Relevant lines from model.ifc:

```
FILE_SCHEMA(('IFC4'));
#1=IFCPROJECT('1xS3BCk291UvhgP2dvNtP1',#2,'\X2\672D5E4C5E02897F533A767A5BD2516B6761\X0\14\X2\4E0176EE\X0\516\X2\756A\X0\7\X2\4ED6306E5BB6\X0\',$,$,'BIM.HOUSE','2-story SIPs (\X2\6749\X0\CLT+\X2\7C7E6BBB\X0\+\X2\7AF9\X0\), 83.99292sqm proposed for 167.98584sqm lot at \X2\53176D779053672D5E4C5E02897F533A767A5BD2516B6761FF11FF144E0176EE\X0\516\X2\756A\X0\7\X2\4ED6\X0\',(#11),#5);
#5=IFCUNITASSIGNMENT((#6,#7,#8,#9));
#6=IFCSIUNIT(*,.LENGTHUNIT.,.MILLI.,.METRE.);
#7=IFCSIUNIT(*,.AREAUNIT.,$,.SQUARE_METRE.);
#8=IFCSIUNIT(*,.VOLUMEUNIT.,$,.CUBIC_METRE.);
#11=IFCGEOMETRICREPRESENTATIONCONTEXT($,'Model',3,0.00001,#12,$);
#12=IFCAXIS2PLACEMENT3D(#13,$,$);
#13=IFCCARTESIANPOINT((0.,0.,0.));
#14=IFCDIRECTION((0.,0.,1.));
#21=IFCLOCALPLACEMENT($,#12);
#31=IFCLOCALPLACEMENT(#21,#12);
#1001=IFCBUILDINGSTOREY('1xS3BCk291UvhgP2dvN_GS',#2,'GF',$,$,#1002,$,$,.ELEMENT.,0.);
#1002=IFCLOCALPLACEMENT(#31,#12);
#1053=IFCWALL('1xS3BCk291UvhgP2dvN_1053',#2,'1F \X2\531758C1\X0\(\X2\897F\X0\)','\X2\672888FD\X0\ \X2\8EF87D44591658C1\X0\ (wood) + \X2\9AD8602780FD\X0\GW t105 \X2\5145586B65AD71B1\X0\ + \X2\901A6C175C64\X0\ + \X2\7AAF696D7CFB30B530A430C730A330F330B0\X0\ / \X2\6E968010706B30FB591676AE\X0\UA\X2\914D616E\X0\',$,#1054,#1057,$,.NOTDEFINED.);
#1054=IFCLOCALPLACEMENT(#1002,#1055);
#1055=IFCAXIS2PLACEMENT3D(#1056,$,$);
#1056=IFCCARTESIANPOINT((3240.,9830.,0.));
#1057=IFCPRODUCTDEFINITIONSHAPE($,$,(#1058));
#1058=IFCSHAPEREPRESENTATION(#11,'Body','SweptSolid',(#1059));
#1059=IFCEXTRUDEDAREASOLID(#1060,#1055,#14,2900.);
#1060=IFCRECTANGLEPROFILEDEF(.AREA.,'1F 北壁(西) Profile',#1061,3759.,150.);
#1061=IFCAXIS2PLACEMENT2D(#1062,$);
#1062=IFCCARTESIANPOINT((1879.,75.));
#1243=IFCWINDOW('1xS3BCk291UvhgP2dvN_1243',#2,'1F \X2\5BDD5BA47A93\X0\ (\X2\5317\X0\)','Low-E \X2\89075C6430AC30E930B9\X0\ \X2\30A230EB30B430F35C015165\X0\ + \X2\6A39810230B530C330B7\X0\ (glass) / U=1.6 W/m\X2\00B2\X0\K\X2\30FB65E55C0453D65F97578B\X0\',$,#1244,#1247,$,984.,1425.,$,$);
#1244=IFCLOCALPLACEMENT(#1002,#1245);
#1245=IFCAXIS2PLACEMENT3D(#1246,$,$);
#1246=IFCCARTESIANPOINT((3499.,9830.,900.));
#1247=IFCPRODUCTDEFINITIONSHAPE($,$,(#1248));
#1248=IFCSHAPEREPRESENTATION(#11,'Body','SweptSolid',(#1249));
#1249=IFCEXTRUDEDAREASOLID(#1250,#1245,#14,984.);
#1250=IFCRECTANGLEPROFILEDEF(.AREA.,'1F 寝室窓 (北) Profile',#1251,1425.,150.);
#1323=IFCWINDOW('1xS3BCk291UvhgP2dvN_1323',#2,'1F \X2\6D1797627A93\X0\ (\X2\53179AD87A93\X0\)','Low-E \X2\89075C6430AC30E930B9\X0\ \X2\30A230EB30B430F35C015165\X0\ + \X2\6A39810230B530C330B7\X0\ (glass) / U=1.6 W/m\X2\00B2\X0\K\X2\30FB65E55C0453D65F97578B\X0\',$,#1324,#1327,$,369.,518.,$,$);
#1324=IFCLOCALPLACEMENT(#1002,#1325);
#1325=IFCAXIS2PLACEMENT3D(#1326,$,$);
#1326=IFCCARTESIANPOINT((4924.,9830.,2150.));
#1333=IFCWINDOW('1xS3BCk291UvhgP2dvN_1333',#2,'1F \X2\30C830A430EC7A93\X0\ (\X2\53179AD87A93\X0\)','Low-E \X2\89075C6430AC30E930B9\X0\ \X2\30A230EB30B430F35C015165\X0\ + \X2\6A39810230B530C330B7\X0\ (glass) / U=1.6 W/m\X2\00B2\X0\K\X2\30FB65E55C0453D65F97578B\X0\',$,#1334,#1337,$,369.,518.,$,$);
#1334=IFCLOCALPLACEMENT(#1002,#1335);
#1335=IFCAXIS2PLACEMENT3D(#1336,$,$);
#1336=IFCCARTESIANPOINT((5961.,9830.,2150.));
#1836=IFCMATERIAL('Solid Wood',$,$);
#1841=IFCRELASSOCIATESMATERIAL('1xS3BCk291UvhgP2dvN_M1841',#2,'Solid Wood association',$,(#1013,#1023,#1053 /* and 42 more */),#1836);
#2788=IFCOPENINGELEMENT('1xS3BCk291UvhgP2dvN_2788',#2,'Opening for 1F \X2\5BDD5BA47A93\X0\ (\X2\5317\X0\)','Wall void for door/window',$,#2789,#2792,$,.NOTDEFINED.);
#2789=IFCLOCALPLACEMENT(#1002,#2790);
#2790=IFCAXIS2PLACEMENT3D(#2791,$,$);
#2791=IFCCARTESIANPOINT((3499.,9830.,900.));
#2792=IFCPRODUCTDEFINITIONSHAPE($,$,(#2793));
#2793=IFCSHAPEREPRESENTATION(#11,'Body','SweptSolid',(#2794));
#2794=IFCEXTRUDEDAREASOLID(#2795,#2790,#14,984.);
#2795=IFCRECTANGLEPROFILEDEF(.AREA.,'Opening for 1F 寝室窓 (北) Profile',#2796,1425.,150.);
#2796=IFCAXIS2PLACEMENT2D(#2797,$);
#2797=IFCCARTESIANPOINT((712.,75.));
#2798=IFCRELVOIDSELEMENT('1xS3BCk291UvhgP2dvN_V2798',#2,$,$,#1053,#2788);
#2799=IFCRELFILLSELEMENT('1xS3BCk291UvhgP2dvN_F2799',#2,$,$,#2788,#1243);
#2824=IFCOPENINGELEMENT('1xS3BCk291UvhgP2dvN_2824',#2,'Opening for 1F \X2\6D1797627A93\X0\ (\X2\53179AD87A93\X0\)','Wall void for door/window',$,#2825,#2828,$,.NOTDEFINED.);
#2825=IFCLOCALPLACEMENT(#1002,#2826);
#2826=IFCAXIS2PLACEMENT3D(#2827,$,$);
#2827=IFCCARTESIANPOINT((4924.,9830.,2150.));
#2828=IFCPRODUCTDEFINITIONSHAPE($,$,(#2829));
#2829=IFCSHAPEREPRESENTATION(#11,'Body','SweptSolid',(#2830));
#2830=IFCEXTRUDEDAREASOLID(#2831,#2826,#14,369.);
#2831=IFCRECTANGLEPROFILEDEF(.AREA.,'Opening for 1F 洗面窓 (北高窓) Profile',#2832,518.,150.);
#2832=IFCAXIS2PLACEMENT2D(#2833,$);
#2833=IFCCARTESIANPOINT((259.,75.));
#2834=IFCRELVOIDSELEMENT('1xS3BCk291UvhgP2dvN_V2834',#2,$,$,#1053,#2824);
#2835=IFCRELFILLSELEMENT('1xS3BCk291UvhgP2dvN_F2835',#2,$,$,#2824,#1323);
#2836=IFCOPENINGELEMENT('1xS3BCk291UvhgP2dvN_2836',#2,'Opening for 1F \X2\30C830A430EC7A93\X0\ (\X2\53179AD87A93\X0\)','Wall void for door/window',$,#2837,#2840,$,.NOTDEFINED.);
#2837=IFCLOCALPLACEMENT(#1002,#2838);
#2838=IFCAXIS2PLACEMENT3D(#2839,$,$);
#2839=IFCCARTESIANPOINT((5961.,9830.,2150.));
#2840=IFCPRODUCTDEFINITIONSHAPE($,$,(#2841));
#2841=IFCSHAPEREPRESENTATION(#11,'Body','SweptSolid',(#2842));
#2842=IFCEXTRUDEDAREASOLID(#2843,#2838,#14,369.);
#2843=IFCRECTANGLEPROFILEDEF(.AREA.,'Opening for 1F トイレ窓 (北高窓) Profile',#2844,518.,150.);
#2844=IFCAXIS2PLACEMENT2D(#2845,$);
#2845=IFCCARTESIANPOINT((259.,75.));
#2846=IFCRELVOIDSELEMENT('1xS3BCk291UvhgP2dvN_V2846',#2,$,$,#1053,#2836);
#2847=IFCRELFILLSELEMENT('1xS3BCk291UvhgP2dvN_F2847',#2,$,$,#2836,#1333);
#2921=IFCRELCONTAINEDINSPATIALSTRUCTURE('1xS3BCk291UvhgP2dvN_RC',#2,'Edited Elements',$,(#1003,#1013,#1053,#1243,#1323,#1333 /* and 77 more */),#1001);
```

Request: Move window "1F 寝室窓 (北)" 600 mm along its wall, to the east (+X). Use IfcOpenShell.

```python
import ifcopenshell
import ifcopenshell.api.geometry
import ifcopenshell.util.placement

model = ifcopenshell.open("model.ifc")

window = model.by_id(1243)
opening = window.FillsVoids[0].RelatingOpeningElement
wall = opening.VoidsElements[0].RelatingBuildingElement

wall_matrix = ifcopenshell.util.placement.get_local_placement(wall.ObjectPlacement)
shift = wall_matrix[:3, 0] * 600.0
before = ifcopenshell.util.placement.get_local_placement(window.ObjectPlacement)[:3, 3].copy()

# The window is not placed relative to its opening, so move both.
for product in (opening, window):
    matrix = ifcopenshell.util.placement.get_local_placement(product.ObjectPlacement)
    matrix[:3, 3] += shift
    ifcopenshell.api.geometry.edit_object_placement(model, product=product, matrix=matrix, is_si=False)

after = ifcopenshell.util.placement.get_local_placement(window.ObjectPlacement)[:3, 3]
print("window moved by", (after - before).round(3) + 0.0)

model.write("model_edited.ifc")
```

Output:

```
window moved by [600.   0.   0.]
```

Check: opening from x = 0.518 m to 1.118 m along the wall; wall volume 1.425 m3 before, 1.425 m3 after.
